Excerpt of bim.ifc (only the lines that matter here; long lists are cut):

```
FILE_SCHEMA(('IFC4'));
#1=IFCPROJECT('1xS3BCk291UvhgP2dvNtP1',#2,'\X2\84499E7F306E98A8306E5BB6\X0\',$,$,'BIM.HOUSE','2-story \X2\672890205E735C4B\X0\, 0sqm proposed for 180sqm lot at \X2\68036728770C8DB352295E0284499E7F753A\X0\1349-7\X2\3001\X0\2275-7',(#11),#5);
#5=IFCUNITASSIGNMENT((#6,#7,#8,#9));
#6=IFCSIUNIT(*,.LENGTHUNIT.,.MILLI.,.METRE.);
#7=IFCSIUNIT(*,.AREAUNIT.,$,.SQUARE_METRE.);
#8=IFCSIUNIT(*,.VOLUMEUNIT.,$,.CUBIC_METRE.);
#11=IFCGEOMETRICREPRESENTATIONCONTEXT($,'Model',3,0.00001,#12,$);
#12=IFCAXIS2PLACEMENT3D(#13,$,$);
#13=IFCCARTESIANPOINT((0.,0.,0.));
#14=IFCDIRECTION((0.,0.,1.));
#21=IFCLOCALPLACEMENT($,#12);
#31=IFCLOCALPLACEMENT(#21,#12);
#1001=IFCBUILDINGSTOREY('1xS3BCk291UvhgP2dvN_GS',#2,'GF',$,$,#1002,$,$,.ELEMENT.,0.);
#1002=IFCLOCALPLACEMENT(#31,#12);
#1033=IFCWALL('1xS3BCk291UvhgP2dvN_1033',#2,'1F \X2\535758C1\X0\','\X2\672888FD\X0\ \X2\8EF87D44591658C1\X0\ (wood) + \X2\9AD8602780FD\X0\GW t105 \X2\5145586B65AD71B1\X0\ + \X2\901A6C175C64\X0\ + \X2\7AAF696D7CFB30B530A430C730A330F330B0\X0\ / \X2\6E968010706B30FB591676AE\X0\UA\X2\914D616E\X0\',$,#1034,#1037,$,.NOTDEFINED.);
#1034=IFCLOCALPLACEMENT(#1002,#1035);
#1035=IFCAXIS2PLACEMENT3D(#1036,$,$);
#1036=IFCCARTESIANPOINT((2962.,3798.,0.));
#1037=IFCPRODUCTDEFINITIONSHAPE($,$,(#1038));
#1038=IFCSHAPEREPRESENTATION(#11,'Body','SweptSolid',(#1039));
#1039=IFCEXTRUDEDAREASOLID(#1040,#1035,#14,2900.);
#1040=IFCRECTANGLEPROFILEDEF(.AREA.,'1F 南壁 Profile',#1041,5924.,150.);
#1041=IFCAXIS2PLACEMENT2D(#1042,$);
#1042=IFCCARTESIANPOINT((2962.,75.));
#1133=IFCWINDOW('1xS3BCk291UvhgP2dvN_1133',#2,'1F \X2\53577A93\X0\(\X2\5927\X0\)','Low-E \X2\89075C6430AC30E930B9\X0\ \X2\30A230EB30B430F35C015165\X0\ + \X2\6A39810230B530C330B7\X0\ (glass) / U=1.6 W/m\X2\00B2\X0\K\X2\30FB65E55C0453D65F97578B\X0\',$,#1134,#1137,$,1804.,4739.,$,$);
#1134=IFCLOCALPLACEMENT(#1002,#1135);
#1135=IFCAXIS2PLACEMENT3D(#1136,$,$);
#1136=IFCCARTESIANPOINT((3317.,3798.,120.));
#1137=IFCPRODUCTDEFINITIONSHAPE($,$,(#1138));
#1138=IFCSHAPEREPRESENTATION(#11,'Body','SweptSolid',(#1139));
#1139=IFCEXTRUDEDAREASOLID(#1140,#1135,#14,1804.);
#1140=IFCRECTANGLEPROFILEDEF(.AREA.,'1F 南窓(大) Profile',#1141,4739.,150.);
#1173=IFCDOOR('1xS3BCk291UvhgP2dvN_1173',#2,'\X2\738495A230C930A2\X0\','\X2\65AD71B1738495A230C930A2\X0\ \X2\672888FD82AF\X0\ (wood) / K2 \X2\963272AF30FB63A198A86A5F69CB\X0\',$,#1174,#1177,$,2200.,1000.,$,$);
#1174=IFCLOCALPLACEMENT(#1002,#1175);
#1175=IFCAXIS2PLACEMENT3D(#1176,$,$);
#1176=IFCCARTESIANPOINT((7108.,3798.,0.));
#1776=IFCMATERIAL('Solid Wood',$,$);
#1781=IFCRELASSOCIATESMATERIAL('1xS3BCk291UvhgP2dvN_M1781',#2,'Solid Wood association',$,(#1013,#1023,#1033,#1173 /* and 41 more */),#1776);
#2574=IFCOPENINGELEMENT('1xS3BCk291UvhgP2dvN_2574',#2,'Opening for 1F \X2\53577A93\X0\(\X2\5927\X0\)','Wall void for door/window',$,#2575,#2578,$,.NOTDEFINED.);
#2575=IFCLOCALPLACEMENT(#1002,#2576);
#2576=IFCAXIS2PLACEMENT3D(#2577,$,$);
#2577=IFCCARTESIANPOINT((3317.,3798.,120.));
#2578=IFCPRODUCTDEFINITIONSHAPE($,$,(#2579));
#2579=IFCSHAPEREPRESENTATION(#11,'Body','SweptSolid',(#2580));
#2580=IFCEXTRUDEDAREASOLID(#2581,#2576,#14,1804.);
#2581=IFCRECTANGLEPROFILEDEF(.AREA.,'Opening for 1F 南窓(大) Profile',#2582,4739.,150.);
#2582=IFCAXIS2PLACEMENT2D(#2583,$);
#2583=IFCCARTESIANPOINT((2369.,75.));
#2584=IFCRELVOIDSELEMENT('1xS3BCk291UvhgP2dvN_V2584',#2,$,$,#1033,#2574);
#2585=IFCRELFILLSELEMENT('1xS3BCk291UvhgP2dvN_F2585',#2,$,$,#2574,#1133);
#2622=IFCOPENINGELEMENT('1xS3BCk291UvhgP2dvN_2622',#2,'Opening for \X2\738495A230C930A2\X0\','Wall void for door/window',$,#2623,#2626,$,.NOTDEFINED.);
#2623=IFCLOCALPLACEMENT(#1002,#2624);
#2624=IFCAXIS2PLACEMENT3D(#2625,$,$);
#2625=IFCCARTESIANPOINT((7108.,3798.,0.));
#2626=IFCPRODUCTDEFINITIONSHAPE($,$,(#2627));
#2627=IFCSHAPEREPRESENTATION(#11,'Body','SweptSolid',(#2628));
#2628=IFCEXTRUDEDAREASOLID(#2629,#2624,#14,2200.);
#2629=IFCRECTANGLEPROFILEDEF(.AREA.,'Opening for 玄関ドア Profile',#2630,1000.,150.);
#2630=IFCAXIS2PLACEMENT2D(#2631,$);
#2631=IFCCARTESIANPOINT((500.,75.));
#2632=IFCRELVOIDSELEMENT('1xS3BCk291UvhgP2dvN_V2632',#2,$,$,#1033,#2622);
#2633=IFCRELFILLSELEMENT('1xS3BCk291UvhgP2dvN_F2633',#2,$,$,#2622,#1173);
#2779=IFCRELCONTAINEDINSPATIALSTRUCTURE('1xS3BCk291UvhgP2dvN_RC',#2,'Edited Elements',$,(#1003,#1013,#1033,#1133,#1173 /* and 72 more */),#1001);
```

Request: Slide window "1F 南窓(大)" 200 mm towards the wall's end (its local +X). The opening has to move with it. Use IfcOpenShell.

```python
import ifcopenshell
import ifcopenshell.api.geometry
import ifcopenshell.util.placement

model = ifcopenshell.open("bim.ifc")

window = model.by_id(1133)
opening = window.FillsVoids[0].RelatingOpeningElement
wall = opening.VoidsElements[0].RelatingBuildingElement

wall_matrix = ifcopenshell.util.placement.get_local_placement(wall.ObjectPlacement)
shift = wall_matrix[:3, 0] * 200.0
before = ifcopenshell.util.placement.get_local_placement(window.ObjectPlacement)[:3, 3].copy()

# The window is not placed relative to its opening, so move both.
for product in (opening, window):
    matrix = ifcopenshell.util.placement.get_local_placement(product.ObjectPlacement)
    matrix[:3, 3] += shift
    ifcopenshell.api.geometry.edit_object_placement(model, product=product, matrix=matrix, is_si=False)

after = ifcopenshell.util.placement.get_local_placement(window.ObjectPlacement)[:3, 3]
print("window moved by", (after - before).round(3) + 0.0)

model.write("bim_rev.ifc")
```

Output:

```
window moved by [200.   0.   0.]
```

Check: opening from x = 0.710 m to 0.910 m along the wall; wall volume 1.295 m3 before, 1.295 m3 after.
